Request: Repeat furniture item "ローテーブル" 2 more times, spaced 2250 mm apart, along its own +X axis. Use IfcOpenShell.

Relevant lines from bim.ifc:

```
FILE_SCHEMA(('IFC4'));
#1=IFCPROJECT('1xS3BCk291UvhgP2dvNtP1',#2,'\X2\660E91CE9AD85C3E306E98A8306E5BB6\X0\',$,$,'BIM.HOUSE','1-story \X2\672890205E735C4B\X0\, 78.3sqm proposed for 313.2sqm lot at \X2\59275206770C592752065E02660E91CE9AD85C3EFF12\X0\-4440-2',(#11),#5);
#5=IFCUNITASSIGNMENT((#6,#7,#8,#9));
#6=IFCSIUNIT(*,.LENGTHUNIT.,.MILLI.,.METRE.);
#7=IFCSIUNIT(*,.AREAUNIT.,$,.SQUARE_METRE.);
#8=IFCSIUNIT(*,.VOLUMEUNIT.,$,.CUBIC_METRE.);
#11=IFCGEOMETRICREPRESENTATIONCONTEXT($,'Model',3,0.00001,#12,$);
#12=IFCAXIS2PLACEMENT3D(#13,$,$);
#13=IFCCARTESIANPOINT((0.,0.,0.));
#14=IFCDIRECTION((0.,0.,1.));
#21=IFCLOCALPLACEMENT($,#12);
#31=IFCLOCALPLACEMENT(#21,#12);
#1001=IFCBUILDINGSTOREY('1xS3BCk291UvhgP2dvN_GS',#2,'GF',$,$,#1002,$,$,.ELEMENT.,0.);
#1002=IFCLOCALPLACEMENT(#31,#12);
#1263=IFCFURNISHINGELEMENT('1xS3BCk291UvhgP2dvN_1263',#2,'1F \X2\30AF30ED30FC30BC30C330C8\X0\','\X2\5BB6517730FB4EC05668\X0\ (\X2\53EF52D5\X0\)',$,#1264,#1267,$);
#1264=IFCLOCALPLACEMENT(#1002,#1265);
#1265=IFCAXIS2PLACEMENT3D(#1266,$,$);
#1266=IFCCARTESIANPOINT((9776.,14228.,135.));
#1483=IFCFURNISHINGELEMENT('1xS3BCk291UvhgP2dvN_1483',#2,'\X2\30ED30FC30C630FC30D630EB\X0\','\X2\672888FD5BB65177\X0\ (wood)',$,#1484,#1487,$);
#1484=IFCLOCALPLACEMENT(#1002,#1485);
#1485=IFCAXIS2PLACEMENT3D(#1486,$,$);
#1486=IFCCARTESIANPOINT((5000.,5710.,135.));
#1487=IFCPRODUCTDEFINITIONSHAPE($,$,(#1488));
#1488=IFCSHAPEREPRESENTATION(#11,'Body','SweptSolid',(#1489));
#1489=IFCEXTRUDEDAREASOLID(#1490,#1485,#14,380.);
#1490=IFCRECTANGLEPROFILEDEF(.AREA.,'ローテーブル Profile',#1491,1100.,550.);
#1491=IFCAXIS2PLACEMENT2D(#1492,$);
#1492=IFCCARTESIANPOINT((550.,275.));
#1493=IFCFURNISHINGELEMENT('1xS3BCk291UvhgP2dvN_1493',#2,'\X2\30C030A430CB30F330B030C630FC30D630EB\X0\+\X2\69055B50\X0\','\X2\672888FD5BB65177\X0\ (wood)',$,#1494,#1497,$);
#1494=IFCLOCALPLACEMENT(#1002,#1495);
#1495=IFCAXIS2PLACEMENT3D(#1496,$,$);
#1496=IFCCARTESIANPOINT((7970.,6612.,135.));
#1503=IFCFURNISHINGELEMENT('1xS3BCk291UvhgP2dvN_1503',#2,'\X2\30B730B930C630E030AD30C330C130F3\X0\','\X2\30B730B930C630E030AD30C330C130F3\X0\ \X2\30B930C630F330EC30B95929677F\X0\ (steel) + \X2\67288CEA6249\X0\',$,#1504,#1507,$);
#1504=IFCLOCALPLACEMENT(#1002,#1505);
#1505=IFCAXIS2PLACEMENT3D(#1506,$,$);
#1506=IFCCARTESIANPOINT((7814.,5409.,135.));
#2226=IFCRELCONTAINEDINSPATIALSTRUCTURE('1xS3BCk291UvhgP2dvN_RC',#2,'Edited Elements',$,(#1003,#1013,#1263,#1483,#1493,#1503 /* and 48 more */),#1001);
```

```python
import ifcopenshell
import ifcopenshell.api.geometry
import ifcopenshell.api.root
import ifcopenshell.util.element
import ifcopenshell.util.placement
import ifcopenshell.util.unit

model = ifcopenshell.open("bim.ifc")
unit_scale = ifcopenshell.util.unit.calculate_unit_scale(model)


def reuse_history(source, copy):
    """copy_class also copies each property set's owner history, people and application; keep the originals."""
    for rel in copy.IsDefinedBy:
        if rel.is_a("IfcRelDefinesByProperties") and (history := rel.RelatingPropertyDefinition.OwnerHistory):
            rel.RelatingPropertyDefinition.OwnerHistory = source.OwnerHistory
            ifcopenshell.util.element.remove_deep2(model, history)


source = model.by_id(1483)
base = ifcopenshell.util.placement.get_local_placement(source.ObjectPlacement)
step = base[:3, 0] * 2.25 / unit_scale

for i in range(1, 3):
    copy = ifcopenshell.api.root.copy_class(model, product=source)
    copy.Representation = ifcopenshell.util.element.copy_deep(
        model, source.Representation, exclude=["IfcGeometricRepresentationContext", "IfcRepresentationMap"]
    )
    reuse_history(source, copy)
    matrix = base.copy()
    matrix[:3, 3] += i * step
    print("added at", matrix[:3, 3].round(3) + 0.0)
    ifcopenshell.api.geometry.edit_object_placement(model, product=copy, matrix=matrix, is_si=False)

model.write("bim_edited.ifc")
```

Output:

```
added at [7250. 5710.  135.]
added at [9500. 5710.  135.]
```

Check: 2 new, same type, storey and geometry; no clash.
